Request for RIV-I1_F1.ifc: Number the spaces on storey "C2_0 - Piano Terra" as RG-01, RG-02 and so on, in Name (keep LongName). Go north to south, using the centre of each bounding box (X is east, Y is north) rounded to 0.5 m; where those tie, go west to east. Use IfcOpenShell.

First a look at what the model holds.

```python
import ifcopenshell
import ifcopenshell.util.element
import ifcopenshell.util.placement

model = ifcopenshell.open("RIV-I1_F1.ifc")
print(model.schema)
storey = next(s for s in model.by_type("IfcBuildingStorey") if s.Name == "C2_0 - Piano Terra")
spaces = [e for e in ifcopenshell.util.element.get_decomposition(storey) if e.is_a("IfcSpace")]
for e in sorted(spaces, key=lambda e: e.id()):
    origin = ifcopenshell.util.placement.get_local_placement(e.ObjectPlacement)[:3, 3]
    print(e.id(), e.Name, e.LongName, origin.round(2) + 0.0, sep=" | ")
```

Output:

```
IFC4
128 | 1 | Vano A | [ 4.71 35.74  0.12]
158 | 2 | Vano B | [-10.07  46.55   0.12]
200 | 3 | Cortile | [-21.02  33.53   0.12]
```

```python
import ifcopenshell
import ifcopenshell.geom
import ifcopenshell.util.element
import ifcopenshell.util.shape

model = ifcopenshell.open("RIV-I1_F1.ifc")
settings = ifcopenshell.geom.settings()
settings.set("use-world-coords", True)


def centre(element):
    shape = ifcopenshell.geom.create_shape(settings, element)
    return ifcopenshell.util.shape.get_bbox_centroid(shape.geometry)


storey = next(s for s in model.by_type("IfcBuildingStorey") if s.Name == "C2_0 - Piano Terra")
spaces = [e for e in ifcopenshell.util.element.get_decomposition(storey) if e.is_a("IfcSpace")]

# Insertion points can sit at a corner or the storey origin, so sort by the geometry (in metres).
centres = {e: centre(e) for e in spaces}
spaces.sort(key=lambda e: (-round(centres[e][1] / 0.5), centres[e][0]))

for i, e in enumerate(spaces, start=1):
    number = f"RG-{i:02d}"
    e.Name = number
    print(e.id(), number)

model.write("RIV-I1_F1_edited.ifc")
```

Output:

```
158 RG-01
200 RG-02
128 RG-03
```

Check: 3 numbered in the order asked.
